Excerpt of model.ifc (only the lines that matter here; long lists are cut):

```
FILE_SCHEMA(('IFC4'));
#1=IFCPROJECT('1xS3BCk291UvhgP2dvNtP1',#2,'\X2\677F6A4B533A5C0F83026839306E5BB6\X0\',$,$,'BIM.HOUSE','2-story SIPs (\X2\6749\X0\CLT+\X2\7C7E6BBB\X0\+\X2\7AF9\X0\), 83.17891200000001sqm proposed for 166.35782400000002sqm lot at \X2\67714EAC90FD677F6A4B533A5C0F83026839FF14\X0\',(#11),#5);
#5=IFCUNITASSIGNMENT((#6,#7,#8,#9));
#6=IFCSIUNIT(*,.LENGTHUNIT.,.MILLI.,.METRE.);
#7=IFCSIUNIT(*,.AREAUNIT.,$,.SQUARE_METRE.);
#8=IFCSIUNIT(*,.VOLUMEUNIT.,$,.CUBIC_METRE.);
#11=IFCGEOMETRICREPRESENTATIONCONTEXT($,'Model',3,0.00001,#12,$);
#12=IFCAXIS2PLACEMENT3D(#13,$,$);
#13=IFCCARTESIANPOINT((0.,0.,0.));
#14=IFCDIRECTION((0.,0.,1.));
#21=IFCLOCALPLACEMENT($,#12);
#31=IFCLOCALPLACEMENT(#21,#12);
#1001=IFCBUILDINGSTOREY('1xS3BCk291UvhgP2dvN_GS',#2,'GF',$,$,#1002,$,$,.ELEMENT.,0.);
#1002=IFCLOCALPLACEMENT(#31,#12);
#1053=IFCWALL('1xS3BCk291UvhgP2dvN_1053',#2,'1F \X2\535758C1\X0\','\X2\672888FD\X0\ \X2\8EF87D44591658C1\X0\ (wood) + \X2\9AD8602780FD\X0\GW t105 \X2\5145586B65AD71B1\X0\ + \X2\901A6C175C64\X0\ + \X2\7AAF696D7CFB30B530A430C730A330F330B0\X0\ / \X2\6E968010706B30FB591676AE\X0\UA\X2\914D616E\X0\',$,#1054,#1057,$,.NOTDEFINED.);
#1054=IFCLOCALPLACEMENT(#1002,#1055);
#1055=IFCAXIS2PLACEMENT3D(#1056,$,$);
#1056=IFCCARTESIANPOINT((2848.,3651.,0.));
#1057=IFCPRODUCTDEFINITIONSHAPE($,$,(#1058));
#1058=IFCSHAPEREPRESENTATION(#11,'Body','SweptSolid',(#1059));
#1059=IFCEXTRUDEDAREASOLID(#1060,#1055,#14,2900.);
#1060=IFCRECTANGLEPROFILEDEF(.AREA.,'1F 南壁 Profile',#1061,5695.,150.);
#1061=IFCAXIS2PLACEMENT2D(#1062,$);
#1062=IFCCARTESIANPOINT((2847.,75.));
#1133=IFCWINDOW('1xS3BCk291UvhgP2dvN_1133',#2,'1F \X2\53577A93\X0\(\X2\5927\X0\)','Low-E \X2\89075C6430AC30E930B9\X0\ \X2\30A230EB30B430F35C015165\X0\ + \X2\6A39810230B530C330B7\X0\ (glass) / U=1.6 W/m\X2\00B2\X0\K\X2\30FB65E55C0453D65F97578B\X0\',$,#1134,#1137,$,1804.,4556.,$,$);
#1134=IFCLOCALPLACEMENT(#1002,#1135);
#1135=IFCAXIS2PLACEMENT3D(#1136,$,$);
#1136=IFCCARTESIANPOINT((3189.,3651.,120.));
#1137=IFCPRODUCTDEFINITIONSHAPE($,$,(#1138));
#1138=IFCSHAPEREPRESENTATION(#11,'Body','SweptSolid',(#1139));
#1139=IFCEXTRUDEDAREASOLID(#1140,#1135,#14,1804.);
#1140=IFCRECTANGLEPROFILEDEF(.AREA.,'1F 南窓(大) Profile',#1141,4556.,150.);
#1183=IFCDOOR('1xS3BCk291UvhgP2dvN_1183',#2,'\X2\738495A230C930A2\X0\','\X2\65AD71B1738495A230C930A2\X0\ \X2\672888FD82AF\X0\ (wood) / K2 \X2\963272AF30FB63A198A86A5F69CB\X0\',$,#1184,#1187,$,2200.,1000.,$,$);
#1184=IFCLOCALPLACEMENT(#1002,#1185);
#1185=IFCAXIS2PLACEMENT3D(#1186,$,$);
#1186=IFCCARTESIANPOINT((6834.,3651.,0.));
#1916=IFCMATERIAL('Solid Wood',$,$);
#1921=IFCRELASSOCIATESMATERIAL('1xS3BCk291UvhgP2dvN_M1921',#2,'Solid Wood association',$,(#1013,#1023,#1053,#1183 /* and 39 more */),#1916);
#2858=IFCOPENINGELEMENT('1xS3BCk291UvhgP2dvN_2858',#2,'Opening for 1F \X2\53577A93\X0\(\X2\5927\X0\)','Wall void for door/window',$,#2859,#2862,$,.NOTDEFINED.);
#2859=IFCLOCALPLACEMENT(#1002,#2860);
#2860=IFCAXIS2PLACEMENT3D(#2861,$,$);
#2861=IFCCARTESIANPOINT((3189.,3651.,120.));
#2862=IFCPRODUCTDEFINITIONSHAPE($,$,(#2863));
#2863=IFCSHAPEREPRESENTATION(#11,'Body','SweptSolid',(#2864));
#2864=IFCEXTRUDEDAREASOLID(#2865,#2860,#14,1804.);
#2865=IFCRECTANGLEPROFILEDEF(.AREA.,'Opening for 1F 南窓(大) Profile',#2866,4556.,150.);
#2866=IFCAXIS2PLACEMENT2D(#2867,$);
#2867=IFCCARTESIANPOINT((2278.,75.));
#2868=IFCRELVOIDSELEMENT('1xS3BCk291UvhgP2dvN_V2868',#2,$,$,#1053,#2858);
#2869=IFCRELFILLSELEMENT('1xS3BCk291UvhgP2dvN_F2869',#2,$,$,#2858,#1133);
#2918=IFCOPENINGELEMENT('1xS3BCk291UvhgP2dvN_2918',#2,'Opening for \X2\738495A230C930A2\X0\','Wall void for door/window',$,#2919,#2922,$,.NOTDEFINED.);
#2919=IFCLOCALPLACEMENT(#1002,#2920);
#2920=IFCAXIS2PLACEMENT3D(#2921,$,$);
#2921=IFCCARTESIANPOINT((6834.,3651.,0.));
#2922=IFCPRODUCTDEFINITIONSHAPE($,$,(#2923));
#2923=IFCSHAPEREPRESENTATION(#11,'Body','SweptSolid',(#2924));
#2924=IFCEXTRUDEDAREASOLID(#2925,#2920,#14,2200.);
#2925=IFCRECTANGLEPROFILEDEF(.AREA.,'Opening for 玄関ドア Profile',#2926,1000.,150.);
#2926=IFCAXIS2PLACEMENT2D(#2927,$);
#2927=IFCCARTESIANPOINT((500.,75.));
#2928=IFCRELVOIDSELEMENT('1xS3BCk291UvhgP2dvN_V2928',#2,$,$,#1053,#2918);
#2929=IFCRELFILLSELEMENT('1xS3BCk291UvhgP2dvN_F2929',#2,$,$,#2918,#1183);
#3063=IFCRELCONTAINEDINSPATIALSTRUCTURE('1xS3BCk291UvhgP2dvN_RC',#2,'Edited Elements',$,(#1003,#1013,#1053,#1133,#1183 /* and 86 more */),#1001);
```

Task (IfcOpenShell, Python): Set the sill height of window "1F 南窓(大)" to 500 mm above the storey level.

```python
import numpy as np
import ifcopenshell
import ifcopenshell.api.geometry
import ifcopenshell.geom
import ifcopenshell.util.element
import ifcopenshell.util.placement
import ifcopenshell.util.shape
import ifcopenshell.util.unit

model = ifcopenshell.open("model.ifc")
unit_scale = ifcopenshell.util.unit.calculate_unit_scale(model)

window = model.by_guid("1xS3BCk291UvhgP2dvN_1133")
opening = window.FillsVoids[0].RelatingOpeningElement
storey = ifcopenshell.util.element.get_container(window, ifc_class="IfcBuildingStorey")
level = ifcopenshell.util.placement.get_local_placement(storey.ObjectPlacement)[2, 3]

# The opening's origin need not be at the sill, so measure its lowest point.
shape = ifcopenshell.geom.create_shape(ifcopenshell.geom.settings(), opening)
bottom = ifcopenshell.util.shape.get_shape_bottom_elevation(shape, shape.geometry) / unit_scale
dz = level + 0.5 / unit_scale - bottom

shift = np.array([0.0, 0.0, dz])
# The window is not placed relative to its opening, so move both.
for product in (opening, window):
    matrix = ifcopenshell.util.placement.get_local_placement(product.ObjectPlacement)
    matrix[:3, 3] += shift
    ifcopenshell.api.geometry.edit_object_placement(model, product=product, matrix=matrix, is_si=False)

print(f"moved by {dz * unit_scale:+.3f} m")

model.write("model_updated.ifc")
```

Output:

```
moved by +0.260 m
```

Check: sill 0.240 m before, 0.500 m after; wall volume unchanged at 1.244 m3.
